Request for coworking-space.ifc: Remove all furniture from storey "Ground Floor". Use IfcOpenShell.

First a look at what the model holds.

```python
import ifcopenshell
import ifcopenshell.util.element

model = ifcopenshell.open("coworking-space.ifc")
print(model.schema)
storey = next(s for s in model.by_type("IfcBuildingStorey") if s.Name == "Ground Floor")
furniture = [e for e in ifcopenshell.util.element.get_decomposition(storey) if e.is_a("IfcFurnishingElement")]
seen = {}
for e in furniture:
    element_type = ifcopenshell.util.element.get_type(e)
    name = element_type.Name if element_type not in (None, e) else None
    seen[name] = seen.get(name, 0) + 1
for name, count in sorted(seen.items(), key=str):
    print(count, "x", name)
```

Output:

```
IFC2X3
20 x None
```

```python
import ifcopenshell
import ifcopenshell.api.root
import ifcopenshell.util.element

model = ifcopenshell.open("coworking-space.ifc")

storey = next(s for s in model.by_type("IfcBuildingStorey") if s.Name == "Ground Floor")
furniture = [e for e in ifcopenshell.util.element.get_decomposition(storey) if e.is_a("IfcFurnishingElement")]

for e in furniture:
    ifcopenshell.api.root.remove_product(model, product=e)
print(len(furniture), "removed")

model.write("coworking-space_edited.ifc")
```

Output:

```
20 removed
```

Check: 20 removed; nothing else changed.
